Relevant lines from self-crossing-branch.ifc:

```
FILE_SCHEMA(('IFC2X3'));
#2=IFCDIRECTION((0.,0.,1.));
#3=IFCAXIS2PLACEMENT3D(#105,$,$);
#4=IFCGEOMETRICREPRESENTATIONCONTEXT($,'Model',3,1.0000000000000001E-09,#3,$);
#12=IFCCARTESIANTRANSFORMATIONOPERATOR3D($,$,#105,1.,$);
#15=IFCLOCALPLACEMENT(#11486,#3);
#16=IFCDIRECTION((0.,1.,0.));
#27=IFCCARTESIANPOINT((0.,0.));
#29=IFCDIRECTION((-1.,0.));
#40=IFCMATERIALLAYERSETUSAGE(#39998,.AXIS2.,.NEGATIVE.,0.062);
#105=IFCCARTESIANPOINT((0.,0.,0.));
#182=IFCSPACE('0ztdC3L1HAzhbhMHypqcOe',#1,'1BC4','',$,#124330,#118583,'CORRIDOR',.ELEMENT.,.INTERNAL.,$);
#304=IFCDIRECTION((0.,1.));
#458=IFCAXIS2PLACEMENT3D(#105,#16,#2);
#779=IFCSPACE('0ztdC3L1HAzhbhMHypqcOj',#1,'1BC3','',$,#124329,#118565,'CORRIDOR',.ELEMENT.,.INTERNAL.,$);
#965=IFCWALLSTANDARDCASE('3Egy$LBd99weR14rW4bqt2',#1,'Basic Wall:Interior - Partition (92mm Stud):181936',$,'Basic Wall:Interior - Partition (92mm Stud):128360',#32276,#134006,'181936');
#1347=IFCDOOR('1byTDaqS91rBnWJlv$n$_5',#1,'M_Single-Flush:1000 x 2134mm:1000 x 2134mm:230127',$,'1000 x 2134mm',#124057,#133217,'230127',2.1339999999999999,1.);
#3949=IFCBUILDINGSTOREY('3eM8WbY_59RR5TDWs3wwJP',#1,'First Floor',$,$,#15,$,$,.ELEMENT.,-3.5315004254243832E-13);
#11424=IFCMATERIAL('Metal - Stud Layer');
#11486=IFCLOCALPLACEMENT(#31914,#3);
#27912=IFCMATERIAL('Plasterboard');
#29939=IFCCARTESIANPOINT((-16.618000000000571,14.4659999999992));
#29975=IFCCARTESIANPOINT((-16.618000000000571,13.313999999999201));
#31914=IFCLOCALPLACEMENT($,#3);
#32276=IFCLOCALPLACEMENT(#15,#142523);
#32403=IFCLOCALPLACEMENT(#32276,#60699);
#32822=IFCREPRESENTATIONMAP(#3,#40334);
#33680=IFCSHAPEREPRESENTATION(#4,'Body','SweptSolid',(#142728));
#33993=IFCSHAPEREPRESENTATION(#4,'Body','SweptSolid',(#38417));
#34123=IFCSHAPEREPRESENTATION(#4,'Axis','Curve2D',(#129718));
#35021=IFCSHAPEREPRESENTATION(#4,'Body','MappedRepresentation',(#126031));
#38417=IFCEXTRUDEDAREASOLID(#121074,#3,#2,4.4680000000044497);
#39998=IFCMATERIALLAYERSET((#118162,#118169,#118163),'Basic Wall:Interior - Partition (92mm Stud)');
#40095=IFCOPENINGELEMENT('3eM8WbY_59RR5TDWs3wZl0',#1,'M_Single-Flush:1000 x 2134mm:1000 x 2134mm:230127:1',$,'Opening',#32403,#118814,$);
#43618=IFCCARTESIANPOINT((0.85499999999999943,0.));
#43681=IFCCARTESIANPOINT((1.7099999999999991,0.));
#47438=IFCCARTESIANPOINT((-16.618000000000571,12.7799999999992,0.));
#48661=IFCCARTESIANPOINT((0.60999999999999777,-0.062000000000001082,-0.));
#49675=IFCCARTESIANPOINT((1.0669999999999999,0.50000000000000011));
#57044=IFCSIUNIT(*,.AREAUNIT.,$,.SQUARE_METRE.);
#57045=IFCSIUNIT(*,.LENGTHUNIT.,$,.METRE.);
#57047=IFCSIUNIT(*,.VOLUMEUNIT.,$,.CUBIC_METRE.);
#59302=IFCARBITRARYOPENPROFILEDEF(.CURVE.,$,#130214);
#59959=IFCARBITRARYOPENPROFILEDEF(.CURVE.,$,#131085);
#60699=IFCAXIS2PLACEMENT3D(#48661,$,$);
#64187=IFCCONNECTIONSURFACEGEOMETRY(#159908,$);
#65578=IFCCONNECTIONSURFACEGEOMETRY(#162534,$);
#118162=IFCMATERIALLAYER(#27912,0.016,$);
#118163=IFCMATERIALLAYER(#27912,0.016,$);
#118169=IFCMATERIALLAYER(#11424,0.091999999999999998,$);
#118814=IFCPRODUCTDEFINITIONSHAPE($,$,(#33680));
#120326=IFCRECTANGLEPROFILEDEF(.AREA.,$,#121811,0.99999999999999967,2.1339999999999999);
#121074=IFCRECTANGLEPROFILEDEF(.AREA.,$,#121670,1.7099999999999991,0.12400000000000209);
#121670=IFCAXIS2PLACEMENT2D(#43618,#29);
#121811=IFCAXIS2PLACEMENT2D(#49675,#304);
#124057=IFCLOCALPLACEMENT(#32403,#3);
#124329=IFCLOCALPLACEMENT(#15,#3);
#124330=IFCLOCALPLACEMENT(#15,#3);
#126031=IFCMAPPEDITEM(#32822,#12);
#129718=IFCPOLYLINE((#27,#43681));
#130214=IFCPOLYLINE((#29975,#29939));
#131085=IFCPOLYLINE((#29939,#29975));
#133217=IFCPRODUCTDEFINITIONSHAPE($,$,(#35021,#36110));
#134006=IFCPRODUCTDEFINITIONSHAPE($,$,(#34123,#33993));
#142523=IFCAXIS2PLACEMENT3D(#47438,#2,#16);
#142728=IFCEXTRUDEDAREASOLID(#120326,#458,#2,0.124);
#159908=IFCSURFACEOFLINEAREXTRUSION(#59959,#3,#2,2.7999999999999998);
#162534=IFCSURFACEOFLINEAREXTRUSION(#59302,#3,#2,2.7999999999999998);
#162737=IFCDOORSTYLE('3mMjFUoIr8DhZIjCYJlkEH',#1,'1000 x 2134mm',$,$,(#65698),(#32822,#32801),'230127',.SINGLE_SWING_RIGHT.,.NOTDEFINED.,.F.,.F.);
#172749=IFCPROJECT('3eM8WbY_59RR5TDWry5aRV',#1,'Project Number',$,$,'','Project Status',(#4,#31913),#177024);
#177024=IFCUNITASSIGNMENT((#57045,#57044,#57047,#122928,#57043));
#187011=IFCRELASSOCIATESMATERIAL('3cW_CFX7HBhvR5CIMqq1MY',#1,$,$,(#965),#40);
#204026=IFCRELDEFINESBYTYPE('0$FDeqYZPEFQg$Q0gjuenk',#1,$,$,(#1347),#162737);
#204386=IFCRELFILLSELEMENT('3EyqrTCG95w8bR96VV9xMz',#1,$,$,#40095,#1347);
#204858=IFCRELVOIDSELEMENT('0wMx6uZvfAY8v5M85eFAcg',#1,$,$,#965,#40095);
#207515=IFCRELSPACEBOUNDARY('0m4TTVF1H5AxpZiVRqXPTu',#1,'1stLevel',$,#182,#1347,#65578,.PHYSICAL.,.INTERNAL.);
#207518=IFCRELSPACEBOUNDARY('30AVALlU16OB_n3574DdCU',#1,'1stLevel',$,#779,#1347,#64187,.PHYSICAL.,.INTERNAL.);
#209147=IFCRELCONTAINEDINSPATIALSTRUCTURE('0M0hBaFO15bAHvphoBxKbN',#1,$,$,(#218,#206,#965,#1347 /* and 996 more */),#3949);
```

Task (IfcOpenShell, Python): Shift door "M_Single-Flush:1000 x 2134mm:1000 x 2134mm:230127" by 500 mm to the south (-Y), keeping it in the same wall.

```python
import numpy as np
import ifcopenshell
import ifcopenshell.api.geometry
import ifcopenshell.util.placement
import ifcopenshell.util.unit

model = ifcopenshell.open("self-crossing-branch.ifc")
unit_scale = ifcopenshell.util.unit.calculate_unit_scale(model)

door = model.by_guid("1byTDaqS91rBnWJlv$n$_5")
opening = door.FillsVoids[0].RelatingOpeningElement
wall = opening.VoidsElements[0].RelatingBuildingElement

wall_matrix = ifcopenshell.util.placement.get_local_placement(wall.ObjectPlacement)
shift = wall_matrix[:3, 0] * -0.5 / unit_scale
before = ifcopenshell.util.placement.get_local_placement(door.ObjectPlacement)[:3, 3].copy()

# The door is placed relative to its opening, so it follows when the opening moves.
matrix = ifcopenshell.util.placement.get_local_placement(opening.ObjectPlacement)
matrix[:3, 3] += shift
ifcopenshell.api.geometry.edit_object_placement(
    model, product=opening, matrix=matrix, is_si=False, should_transform_children=True
)

# Space boundary surfaces are stored in each space's coordinates; move them too.
for rel in door.ProvidesBoundaries:
    if not rel.ConnectionGeometry:
        continue
    surface = rel.ConnectionGeometry.SurfaceOnRelatingElement
    space_matrix = ifcopenshell.util.placement.get_local_placement(rel.RelatingSpace.ObjectPlacement)
    point = np.array(surface.Position.Location.Coordinates) + space_matrix[:3, :3].T @ shift
    surface.Position = model.createIfcAxis2Placement3D(
        model.createIfcCartesianPoint(point.tolist()), surface.Position.Axis, surface.Position.RefDirection
    )

after = ifcopenshell.util.placement.get_local_placement(door.ObjectPlacement)[:3, 3]
print("door moved by", (after - before).round(3) + 0.0)

model.write("self-crossing-branch-out.ifc")
```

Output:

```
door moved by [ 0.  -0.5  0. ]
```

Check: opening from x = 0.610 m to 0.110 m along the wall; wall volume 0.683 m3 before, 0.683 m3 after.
